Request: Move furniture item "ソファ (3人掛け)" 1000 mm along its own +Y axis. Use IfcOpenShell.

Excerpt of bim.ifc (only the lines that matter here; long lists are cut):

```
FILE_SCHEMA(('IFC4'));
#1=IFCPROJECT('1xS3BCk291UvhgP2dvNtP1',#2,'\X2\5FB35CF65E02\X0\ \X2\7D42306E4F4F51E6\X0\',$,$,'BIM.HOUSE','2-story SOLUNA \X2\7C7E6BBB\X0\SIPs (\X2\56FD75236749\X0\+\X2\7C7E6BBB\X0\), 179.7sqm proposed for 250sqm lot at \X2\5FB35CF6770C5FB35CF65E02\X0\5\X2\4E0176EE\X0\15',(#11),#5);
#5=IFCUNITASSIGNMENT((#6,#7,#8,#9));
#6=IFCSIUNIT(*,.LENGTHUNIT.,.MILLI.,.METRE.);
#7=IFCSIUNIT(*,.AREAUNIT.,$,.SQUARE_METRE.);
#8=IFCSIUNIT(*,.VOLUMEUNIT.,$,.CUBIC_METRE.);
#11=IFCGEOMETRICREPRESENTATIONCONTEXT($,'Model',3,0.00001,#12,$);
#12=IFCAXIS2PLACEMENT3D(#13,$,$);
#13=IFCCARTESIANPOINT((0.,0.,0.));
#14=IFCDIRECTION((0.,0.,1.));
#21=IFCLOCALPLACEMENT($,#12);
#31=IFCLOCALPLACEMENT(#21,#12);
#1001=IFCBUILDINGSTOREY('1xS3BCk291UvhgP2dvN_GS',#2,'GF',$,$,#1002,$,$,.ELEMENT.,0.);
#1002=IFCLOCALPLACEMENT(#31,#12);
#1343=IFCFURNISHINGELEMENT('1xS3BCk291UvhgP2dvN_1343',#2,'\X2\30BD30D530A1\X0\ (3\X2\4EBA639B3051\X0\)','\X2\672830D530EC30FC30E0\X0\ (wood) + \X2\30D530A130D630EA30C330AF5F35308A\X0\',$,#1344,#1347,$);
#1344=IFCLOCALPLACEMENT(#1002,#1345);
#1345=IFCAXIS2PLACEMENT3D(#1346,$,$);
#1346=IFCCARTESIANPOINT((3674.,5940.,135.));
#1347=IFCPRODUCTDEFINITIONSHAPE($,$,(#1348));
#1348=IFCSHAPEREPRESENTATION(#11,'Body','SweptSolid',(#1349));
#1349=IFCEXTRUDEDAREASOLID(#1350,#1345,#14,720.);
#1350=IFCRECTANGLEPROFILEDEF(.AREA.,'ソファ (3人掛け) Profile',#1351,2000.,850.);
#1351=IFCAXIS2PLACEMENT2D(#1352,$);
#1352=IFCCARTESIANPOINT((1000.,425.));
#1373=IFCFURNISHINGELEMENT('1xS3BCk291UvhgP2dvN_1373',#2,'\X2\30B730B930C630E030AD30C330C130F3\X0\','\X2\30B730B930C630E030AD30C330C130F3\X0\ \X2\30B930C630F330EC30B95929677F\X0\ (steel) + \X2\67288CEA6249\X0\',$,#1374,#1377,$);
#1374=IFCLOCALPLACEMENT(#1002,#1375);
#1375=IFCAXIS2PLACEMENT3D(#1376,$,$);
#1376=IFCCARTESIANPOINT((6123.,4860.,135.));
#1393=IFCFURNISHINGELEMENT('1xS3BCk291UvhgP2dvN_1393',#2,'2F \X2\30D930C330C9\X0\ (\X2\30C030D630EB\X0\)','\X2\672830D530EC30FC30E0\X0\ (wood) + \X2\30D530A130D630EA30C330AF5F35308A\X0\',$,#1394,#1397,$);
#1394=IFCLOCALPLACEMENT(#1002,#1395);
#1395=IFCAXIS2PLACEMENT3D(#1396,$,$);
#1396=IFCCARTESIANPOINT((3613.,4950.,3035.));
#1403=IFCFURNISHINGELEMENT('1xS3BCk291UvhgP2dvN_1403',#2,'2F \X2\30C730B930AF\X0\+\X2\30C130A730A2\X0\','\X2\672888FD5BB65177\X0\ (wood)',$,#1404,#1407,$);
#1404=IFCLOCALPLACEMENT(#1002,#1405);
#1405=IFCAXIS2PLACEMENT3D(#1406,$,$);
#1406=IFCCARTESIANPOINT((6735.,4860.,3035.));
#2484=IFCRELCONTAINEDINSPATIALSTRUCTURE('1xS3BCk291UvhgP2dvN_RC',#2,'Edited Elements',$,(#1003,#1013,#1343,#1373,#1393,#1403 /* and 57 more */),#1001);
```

```python
import ifcopenshell
import ifcopenshell.api.geometry
import ifcopenshell.util.placement
import ifcopenshell.util.unit

model = ifcopenshell.open("bim.ifc")
unit_scale = ifcopenshell.util.unit.calculate_unit_scale(model)

item = model.by_guid("1xS3BCk291UvhgP2dvN_1343")
matrix = ifcopenshell.util.placement.get_local_placement(item.ObjectPlacement)
matrix[:3, 3] += matrix[:3, 1] * 1 / unit_scale
ifcopenshell.api.geometry.edit_object_placement(model, product=item, matrix=matrix, is_si=False)

print(ifcopenshell.util.placement.get_local_placement(item.ObjectPlacement).round(3) + 0.0)

model.write("bim_updated.ifc")
```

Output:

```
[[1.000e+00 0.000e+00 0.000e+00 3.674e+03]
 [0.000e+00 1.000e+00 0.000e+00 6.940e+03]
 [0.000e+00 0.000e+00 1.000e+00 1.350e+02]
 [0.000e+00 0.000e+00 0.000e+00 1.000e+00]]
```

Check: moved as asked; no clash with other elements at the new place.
